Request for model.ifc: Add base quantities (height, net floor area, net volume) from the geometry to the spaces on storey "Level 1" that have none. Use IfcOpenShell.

First a look at what the model holds.

```python
import ifcopenshell
import ifcopenshell.util.element
import ifcopenshell.util.unit

model = ifcopenshell.open("model.ifc")
print(model.schema)
for unit_type in ("LENGTHUNIT", "AREAUNIT", "VOLUMEUNIT"):
    print(unit_type, ifcopenshell.util.unit.calculate_unit_scale(model, unit_type))
storey = next(s for s in model.by_type("IfcBuildingStorey") if s.Name == "Level 1")
spaces = [e for e in ifcopenshell.util.element.get_decomposition(storey) if e.is_a("IfcSpace")]
for e in sorted(spaces, key=lambda e: e.id()):
    print(e.id(), e.is_a(), e.Name, list(ifcopenshell.util.element.get_psets(e, qtos_only=True)), sep=" | ")
```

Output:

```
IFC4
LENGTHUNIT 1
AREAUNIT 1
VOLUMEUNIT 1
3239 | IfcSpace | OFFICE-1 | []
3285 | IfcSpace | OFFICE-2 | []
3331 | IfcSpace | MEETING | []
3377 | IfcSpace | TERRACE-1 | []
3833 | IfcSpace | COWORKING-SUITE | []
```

```python
import ifcopenshell
import ifcopenshell.api.pset
import ifcopenshell.geom
import ifcopenshell.util.element
import ifcopenshell.util.shape
import ifcopenshell.util.unit

model = ifcopenshell.open("model.ifc")
unit_scale = ifcopenshell.util.unit.calculate_unit_scale(model)
area_scale = ifcopenshell.util.unit.calculate_unit_scale(model, "AREAUNIT")
volume_scale = ifcopenshell.util.unit.calculate_unit_scale(model, "VOLUMEUNIT")
settings = ifcopenshell.geom.settings()

storey = next(s for s in model.by_type("IfcBuildingStorey") if s.Name == "Level 1")
spaces = [e for e in ifcopenshell.util.element.get_decomposition(storey) if e.is_a("IfcSpace")]

for e in sorted(spaces, key=lambda e: e.id()):
    if ifcopenshell.util.element.get_psets(e, qtos_only=True, should_inherit=False):
        continue
    # Geometry comes back in metres, in the element's own axes.
    shape = ifcopenshell.geom.create_shape(settings, e)
    values = {
        "Height": ifcopenshell.util.shape.get_z(shape.geometry) / unit_scale,
        "NetFloorArea": ifcopenshell.util.shape.get_footprint_area(shape.geometry) / area_scale,
        "NetVolume": ifcopenshell.util.shape.get_volume(shape.geometry) / volume_scale,
    }
    qto = ifcopenshell.api.pset.add_qto(model, product=e, name="Qto_SpaceBaseQuantities")
    ifcopenshell.api.pset.edit_qto(model, qto=qto, properties=values)
    print(e.id(), {k: round(v, 3) for k, v in values.items()})

model.write("model_edited.ifc")
```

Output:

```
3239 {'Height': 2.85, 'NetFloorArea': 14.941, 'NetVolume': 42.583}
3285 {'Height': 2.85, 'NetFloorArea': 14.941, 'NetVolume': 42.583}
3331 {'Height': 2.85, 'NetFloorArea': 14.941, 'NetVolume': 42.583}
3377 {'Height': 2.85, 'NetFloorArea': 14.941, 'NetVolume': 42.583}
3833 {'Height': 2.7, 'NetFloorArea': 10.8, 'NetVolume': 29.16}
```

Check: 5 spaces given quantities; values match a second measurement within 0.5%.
